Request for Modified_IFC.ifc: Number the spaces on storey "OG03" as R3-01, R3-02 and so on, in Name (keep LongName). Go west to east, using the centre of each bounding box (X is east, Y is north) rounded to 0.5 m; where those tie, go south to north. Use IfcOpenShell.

First a look at what the model holds.

```python
import ifcopenshell
import ifcopenshell.util.element
import ifcopenshell.util.placement

model = ifcopenshell.open("Modified_IFC.ifc")
print(model.schema)
storey = next(s for s in model.by_type("IfcBuildingStorey") if s.Name == "OG03")
spaces = [e for e in ifcopenshell.util.element.get_decomposition(storey) if e.is_a("IfcSpace")]
for e in sorted(spaces, key=lambda e: e.id()):
    origin = ifcopenshell.util.placement.get_local_placement(e.ObjectPlacement)[:3, 3]
    print(e.id(), e.Name, e.LongName, origin.round(2) + 0.0, sep=" | ")
```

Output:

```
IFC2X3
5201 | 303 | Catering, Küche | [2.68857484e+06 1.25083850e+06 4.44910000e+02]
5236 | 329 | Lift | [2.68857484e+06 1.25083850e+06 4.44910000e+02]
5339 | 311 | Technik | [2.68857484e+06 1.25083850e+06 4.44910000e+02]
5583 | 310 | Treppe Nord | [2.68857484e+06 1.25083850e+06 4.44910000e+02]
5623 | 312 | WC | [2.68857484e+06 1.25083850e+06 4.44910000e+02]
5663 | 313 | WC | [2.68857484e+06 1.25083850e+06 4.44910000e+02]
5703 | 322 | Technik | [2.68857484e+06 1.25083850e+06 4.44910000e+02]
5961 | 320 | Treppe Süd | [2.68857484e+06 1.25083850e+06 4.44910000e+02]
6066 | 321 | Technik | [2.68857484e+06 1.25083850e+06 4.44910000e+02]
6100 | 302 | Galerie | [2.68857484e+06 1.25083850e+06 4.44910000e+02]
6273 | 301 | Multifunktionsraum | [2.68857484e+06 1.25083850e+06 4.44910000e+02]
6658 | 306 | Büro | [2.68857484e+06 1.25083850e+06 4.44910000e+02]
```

```python
import ifcopenshell
import ifcopenshell.geom
import ifcopenshell.util.element
import ifcopenshell.util.shape

model = ifcopenshell.open("Modified_IFC.ifc")
settings = ifcopenshell.geom.settings()
settings.set("use-world-coords", True)


def centre(element):
    shape = ifcopenshell.geom.create_shape(settings, element)
    return ifcopenshell.util.shape.get_bbox_centroid(shape.geometry)


storey = next(s for s in model.by_type("IfcBuildingStorey") if s.Name == "OG03")
spaces = [e for e in ifcopenshell.util.element.get_decomposition(storey) if e.is_a("IfcSpace")]

# Insertion points can sit at a corner or the storey origin, so sort by the geometry (in metres).
centres = {e: centre(e) for e in spaces}
spaces.sort(key=lambda e: (round(centres[e][0] / 0.5), centres[e][1]))

for i, e in enumerate(spaces, start=1):
    number = f"R3-{i:02d}"
    e.Name = number
    print(e.id(), number)

model.write("Modified_IFC_v2.ifc")
```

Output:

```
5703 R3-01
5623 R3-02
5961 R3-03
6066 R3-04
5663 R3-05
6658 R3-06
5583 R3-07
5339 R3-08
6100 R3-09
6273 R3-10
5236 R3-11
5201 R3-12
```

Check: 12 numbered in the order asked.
